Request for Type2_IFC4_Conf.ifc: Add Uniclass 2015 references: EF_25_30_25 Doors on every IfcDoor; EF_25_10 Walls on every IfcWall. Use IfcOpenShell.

First a look at what the model holds.

```python
import ifcopenshell

model = ifcopenshell.open("Type2_IFC4_Conf.ifc")
print(model.schema)
print("classifications:", [c.Name for c in model.by_type("IfcClassification")])
for ifc_class in ("IfcDoor", "IfcRoof", "IfcStair", "IfcWall", "IfcWindow"):
    print(ifc_class, len(model.by_type(ifc_class)))
```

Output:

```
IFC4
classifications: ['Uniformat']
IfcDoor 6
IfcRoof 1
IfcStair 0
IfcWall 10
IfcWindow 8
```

```python
import ifcopenshell
import ifcopenshell.api.classification

model = ifcopenshell.open("Type2_IFC4_Conf.ifc")

system = ifcopenshell.api.classification.add_classification(model, classification="Uniclass 2015")

codes = {
    "IfcDoor": ("EF_25_30_25", "Doors"),
    "IfcWall": ("EF_25_10", "Walls"),
}
for ifc_class, (code, name) in codes.items():
    products = model.by_type(ifc_class)
    ifcopenshell.api.classification.add_reference(
        model, products=products, classification=system, identification=code, name=name
    )
    print(code, len(products))

model.write("Type2_IFC4_Conf-out.ifc")
```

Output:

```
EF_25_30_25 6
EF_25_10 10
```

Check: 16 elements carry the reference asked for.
